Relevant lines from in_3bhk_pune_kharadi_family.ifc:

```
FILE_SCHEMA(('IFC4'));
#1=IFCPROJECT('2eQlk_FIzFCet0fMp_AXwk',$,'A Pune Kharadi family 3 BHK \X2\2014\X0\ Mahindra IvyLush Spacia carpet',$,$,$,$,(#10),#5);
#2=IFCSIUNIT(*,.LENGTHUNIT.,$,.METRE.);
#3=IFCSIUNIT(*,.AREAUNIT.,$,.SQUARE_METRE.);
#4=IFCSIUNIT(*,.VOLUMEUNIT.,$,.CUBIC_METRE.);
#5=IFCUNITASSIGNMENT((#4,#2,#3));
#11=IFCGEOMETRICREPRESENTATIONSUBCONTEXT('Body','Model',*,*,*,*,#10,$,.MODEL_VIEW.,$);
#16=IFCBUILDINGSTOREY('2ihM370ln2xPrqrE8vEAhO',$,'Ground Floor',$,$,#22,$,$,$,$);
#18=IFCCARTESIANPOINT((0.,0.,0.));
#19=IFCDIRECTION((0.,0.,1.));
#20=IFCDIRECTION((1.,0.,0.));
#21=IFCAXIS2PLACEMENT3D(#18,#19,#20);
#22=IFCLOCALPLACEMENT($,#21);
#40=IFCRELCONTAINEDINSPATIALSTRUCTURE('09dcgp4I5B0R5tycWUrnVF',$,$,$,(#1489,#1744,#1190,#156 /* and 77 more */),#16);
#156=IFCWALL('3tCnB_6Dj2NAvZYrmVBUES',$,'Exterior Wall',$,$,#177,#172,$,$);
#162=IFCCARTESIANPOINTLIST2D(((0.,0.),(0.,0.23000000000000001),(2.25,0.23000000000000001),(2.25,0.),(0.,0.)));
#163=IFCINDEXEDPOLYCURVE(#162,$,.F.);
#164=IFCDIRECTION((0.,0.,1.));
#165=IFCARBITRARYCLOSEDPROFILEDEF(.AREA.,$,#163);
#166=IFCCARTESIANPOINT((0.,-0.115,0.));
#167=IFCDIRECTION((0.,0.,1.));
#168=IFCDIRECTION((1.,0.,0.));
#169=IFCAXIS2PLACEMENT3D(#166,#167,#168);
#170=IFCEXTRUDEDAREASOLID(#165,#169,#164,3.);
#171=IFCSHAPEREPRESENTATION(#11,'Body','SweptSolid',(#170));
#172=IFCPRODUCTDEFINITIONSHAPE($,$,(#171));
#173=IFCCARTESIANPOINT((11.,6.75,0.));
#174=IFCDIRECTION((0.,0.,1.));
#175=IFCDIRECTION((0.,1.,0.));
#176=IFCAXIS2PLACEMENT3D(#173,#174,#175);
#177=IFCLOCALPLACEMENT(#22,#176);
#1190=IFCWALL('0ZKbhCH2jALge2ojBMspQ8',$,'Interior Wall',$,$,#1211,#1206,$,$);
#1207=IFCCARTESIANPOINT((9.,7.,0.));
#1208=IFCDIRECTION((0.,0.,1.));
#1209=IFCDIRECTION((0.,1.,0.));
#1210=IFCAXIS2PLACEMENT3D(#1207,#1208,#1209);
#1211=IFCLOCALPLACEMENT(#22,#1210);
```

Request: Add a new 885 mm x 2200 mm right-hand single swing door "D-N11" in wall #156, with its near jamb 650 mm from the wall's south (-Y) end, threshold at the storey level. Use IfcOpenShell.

```python
import numpy as np
import ifcopenshell
import ifcopenshell.api.feature
import ifcopenshell.api.geometry
import ifcopenshell.api.root
import ifcopenshell.api.spatial
import ifcopenshell.geom
import ifcopenshell.util.element
import ifcopenshell.util.placement
import ifcopenshell.util.representation
import ifcopenshell.util.shape
import ifcopenshell.util.unit

model = ifcopenshell.open("in_3bhk_pune_kharadi_family.ifc")
unit_scale = ifcopenshell.util.unit.calculate_unit_scale(model)
settings = ifcopenshell.geom.settings()


def volume(element):
    """Net volume in cubic metres, openings subtracted."""
    shape = ifcopenshell.geom.create_shape(settings, element)
    return ifcopenshell.util.shape.get_volume(shape.geometry)


wall = model.by_id(156)
storey = ifcopenshell.util.element.get_container(wall, ifc_class="IfcBuildingStorey")
context = ifcopenshell.util.representation.get_context(model, "Model", "Body", "MODEL_VIEW")
before = volume(wall)

width, height, from_end, sill = 0.885, 2.2, 0.65, 0.0  # metres

# The wall runs along its own X axis, and the end named is its -X end.
wall_shape = ifcopenshell.geom.create_shape(settings, wall)
x, y, z = ifcopenshell.util.shape.get_vertices(wall_shape.geometry).T
start = x.min() + from_end
face, thickness = float(y.min()), float(y.max() - y.min())
wall_matrix = ifcopenshell.util.placement.get_local_placement(wall.ObjectPlacement)
level = ifcopenshell.util.placement.get_local_placement(storey.ObjectPlacement)[2, 3]


def in_wall(x, y):
    """Placement at x, y metres in the wall's axes, at sill height."""
    matrix = wall_matrix.copy()
    matrix[:, 3] = wall_matrix @ np.array([x / unit_scale, y / unit_scale, 0.0, 1.0])
    matrix[2, 3] = level + sill / unit_scale
    return matrix


# Opening: a box that overshoots both wall faces by 50 mm.
opening = ifcopenshell.api.root.create_entity(model, ifc_class="IfcOpeningElement", predefined_type="OPENING")
box = ifcopenshell.api.geometry.add_wall_representation(
    model, context=context, length=width, height=height, thickness=thickness + 0.1
)
ifcopenshell.api.geometry.assign_representation(model, product=opening, representation=box)
ifcopenshell.api.geometry.edit_object_placement(model, product=opening, matrix=in_wall(start, face - 0.05), is_si=False)
ifcopenshell.api.feature.add_feature(model, feature=opening, element=wall)

door = ifcopenshell.api.root.create_entity(model, ifc_class="IfcDoor", name="D-N11", predefined_type="DOOR")
door.OverallWidth, door.OverallHeight = width / unit_scale, height / unit_scale
door.OperationType = "SINGLE_SWING_RIGHT"
body = ifcopenshell.api.geometry.add_door_representation(
    model,
    context=context,
    overall_width=door.OverallWidth,
    overall_height=door.OverallHeight,
    operation_type="SINGLE_SWING_RIGHT",
    lining_properties={"LiningDepth": thickness / unit_scale, "ThresholdDepth": thickness / unit_scale},
)
ifcopenshell.api.geometry.assign_representation(model, product=door, representation=body)
ifcopenshell.api.spatial.assign_container(model, products=[door], relating_structure=storey)
ifcopenshell.api.feature.add_filling(model, opening=opening, element=door)

# The lining spans the wall, so the door starts at the wall face.
ifcopenshell.api.geometry.edit_object_placement(model, product=door, matrix=in_wall(start, face), is_si=False)

after = volume(wall)

print(f"wall volume {before:.3f} -> {after:.3f} m3")

model.write("in_3bhk_pune_kharadi_family-out.ifc")
```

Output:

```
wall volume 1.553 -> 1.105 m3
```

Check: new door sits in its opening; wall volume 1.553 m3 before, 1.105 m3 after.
